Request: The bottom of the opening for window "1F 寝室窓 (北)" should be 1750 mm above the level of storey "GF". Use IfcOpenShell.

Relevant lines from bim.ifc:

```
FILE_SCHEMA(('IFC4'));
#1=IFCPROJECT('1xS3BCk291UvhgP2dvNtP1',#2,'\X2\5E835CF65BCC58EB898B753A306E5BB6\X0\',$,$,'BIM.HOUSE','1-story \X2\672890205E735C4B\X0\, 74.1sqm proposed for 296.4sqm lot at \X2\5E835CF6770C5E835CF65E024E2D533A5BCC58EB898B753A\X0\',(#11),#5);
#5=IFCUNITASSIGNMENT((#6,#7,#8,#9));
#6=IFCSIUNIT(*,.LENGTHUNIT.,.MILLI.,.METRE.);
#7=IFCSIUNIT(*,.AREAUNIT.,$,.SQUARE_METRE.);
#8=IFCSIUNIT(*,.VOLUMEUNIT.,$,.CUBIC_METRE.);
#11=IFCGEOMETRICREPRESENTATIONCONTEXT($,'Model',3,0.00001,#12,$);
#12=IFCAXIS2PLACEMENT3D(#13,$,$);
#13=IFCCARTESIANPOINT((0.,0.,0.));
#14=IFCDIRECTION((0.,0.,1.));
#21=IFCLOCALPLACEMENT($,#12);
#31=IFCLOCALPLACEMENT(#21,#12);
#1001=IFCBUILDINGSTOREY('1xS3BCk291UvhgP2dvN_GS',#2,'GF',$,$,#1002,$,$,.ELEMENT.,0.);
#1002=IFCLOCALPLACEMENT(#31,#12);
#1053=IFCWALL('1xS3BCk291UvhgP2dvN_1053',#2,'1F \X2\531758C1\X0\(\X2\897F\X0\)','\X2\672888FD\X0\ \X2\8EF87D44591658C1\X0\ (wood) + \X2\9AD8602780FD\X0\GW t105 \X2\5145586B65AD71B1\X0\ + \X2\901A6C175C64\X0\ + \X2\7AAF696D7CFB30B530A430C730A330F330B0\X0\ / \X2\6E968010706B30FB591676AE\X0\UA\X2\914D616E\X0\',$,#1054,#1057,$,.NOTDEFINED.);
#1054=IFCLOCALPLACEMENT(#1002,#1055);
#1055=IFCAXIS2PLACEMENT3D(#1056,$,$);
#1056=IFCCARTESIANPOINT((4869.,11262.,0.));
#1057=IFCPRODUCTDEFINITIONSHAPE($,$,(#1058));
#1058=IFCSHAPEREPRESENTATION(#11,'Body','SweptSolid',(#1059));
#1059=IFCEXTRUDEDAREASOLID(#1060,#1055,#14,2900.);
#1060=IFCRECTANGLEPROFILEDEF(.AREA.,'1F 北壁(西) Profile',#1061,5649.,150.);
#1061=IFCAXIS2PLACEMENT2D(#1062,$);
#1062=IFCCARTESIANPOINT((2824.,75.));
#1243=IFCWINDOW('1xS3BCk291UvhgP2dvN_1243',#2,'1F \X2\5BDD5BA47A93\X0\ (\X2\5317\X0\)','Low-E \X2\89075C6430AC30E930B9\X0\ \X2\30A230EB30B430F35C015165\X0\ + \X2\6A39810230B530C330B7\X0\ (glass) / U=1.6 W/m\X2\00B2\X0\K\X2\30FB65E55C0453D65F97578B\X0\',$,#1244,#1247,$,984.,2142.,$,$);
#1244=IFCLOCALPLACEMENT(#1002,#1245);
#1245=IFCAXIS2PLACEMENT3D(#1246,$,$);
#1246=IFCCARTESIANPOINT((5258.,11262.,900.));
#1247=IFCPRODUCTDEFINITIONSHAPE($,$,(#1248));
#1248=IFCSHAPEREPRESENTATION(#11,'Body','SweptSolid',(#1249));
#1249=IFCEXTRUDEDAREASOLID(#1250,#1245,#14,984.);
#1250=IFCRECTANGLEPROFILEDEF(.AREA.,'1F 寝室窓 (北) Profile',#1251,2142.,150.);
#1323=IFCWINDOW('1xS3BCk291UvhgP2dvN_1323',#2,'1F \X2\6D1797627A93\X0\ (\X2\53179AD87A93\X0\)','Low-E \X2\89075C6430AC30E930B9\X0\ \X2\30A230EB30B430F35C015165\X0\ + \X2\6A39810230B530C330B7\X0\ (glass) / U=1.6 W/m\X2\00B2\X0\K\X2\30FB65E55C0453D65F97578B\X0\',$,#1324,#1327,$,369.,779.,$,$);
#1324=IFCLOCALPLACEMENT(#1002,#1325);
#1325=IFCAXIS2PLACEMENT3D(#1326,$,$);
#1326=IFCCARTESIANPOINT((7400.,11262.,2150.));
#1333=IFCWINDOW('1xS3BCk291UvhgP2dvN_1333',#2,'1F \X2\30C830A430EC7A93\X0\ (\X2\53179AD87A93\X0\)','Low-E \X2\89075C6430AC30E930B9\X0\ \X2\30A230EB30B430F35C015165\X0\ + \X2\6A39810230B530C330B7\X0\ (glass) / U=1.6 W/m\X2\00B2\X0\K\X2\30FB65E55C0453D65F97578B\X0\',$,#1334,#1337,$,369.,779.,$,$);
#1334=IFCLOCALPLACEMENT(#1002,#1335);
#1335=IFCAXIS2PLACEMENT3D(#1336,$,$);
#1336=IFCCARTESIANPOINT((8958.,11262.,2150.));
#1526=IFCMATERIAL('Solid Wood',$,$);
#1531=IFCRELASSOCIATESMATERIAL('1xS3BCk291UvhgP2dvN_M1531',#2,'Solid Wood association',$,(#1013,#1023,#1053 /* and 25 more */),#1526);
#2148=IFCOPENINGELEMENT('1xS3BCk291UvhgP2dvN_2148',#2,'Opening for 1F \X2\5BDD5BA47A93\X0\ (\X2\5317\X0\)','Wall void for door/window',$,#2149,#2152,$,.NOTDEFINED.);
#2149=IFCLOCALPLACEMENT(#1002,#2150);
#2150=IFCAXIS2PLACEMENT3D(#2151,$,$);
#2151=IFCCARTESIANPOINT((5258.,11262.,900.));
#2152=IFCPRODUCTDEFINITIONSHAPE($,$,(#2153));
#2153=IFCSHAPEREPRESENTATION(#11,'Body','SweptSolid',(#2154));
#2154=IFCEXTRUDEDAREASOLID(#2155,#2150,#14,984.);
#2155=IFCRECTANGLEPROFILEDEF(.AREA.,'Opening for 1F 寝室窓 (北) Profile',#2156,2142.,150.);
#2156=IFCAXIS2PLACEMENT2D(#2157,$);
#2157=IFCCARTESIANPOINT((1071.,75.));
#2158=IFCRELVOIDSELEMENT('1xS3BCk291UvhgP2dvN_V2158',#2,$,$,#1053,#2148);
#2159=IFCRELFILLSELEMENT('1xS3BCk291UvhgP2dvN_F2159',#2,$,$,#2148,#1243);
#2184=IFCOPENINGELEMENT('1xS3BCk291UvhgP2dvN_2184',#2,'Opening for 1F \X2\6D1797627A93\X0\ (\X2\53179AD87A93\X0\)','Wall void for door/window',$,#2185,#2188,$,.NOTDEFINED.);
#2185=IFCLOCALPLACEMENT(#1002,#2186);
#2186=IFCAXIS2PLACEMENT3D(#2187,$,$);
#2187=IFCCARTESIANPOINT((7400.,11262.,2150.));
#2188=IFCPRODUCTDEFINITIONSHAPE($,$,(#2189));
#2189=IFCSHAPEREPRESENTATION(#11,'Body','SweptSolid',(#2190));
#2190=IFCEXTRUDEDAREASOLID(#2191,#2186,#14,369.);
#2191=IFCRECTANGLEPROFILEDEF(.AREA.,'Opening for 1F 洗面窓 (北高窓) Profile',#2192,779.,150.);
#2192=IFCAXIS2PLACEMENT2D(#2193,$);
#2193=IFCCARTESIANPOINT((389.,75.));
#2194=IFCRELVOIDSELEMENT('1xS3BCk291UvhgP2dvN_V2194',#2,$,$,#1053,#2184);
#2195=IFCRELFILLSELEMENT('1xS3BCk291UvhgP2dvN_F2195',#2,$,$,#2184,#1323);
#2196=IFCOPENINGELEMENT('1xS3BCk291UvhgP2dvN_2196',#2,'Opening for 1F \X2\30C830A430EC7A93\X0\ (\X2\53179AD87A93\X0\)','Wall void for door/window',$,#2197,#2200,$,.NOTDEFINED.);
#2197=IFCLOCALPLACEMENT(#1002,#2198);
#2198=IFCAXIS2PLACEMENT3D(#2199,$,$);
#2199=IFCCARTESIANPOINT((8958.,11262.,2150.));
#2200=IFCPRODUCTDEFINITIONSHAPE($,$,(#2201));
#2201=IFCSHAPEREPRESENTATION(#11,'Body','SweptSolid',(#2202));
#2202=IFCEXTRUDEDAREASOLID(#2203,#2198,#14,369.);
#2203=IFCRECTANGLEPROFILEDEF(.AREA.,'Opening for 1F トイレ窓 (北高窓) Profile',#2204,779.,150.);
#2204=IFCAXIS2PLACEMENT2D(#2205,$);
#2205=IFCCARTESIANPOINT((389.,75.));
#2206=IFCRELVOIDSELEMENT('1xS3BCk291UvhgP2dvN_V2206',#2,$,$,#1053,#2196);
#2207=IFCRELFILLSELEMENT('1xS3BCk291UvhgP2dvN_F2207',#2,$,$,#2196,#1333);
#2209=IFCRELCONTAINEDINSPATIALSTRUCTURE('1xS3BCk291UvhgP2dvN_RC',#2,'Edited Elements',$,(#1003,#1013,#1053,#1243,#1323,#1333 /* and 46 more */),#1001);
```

```python
import numpy as np
import ifcopenshell
import ifcopenshell.api.geometry
import ifcopenshell.geom
import ifcopenshell.util.element
import ifcopenshell.util.placement
import ifcopenshell.util.shape
import ifcopenshell.util.unit

model = ifcopenshell.open("bim.ifc")
unit_scale = ifcopenshell.util.unit.calculate_unit_scale(model)

window = model.by_id(1243)
opening = window.FillsVoids[0].RelatingOpeningElement
storey = ifcopenshell.util.element.get_container(window, ifc_class="IfcBuildingStorey")
level = ifcopenshell.util.placement.get_local_placement(storey.ObjectPlacement)[2, 3]

# The opening's origin need not be at the sill, so measure its lowest point.
shape = ifcopenshell.geom.create_shape(ifcopenshell.geom.settings(), opening)
bottom = ifcopenshell.util.shape.get_shape_bottom_elevation(shape, shape.geometry) / unit_scale
dz = level + 1750.0 - bottom

shift = np.array([0.0, 0.0, dz])
# The window is not placed relative to its opening, so move both.
for product in (opening, window):
    matrix = ifcopenshell.util.placement.get_local_placement(product.ObjectPlacement)
    matrix[:3, 3] += shift
    ifcopenshell.api.geometry.edit_object_placement(model, product=product, matrix=matrix, is_si=False)

print(f"moved by {dz * unit_scale:+.3f} m")

model.write("bim_updated.ifc")
```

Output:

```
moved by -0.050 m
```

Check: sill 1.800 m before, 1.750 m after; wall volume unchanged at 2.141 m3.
